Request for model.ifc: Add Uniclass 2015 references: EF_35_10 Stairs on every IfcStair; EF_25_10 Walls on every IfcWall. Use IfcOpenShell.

First a look at what the model holds.

```python
import ifcopenshell

model = ifcopenshell.open("model.ifc")
print(model.schema)
print("classifications:", [c.Name for c in model.by_type("IfcClassification")])
for ifc_class in ("IfcDoor", "IfcRoof", "IfcStair", "IfcWall", "IfcWindow"):
    print(ifc_class, len(model.by_type(ifc_class)))
```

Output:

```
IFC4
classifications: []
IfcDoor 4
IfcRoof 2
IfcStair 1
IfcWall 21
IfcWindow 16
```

```python
import ifcopenshell
import ifcopenshell.api.classification

model = ifcopenshell.open("model.ifc")

system = ifcopenshell.api.classification.add_classification(model, classification="Uniclass 2015")

codes = {
    "IfcStair": ("EF_35_10", "Stairs"),
    "IfcWall": ("EF_25_10", "Walls"),
}
for ifc_class, (code, name) in codes.items():
    products = model.by_type(ifc_class)
    ifcopenshell.api.classification.add_reference(
        model, products=products, classification=system, identification=code, name=name
    )
    print(code, len(products))

model.write("model_updated.ifc")
```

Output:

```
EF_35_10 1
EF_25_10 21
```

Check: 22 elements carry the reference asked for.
